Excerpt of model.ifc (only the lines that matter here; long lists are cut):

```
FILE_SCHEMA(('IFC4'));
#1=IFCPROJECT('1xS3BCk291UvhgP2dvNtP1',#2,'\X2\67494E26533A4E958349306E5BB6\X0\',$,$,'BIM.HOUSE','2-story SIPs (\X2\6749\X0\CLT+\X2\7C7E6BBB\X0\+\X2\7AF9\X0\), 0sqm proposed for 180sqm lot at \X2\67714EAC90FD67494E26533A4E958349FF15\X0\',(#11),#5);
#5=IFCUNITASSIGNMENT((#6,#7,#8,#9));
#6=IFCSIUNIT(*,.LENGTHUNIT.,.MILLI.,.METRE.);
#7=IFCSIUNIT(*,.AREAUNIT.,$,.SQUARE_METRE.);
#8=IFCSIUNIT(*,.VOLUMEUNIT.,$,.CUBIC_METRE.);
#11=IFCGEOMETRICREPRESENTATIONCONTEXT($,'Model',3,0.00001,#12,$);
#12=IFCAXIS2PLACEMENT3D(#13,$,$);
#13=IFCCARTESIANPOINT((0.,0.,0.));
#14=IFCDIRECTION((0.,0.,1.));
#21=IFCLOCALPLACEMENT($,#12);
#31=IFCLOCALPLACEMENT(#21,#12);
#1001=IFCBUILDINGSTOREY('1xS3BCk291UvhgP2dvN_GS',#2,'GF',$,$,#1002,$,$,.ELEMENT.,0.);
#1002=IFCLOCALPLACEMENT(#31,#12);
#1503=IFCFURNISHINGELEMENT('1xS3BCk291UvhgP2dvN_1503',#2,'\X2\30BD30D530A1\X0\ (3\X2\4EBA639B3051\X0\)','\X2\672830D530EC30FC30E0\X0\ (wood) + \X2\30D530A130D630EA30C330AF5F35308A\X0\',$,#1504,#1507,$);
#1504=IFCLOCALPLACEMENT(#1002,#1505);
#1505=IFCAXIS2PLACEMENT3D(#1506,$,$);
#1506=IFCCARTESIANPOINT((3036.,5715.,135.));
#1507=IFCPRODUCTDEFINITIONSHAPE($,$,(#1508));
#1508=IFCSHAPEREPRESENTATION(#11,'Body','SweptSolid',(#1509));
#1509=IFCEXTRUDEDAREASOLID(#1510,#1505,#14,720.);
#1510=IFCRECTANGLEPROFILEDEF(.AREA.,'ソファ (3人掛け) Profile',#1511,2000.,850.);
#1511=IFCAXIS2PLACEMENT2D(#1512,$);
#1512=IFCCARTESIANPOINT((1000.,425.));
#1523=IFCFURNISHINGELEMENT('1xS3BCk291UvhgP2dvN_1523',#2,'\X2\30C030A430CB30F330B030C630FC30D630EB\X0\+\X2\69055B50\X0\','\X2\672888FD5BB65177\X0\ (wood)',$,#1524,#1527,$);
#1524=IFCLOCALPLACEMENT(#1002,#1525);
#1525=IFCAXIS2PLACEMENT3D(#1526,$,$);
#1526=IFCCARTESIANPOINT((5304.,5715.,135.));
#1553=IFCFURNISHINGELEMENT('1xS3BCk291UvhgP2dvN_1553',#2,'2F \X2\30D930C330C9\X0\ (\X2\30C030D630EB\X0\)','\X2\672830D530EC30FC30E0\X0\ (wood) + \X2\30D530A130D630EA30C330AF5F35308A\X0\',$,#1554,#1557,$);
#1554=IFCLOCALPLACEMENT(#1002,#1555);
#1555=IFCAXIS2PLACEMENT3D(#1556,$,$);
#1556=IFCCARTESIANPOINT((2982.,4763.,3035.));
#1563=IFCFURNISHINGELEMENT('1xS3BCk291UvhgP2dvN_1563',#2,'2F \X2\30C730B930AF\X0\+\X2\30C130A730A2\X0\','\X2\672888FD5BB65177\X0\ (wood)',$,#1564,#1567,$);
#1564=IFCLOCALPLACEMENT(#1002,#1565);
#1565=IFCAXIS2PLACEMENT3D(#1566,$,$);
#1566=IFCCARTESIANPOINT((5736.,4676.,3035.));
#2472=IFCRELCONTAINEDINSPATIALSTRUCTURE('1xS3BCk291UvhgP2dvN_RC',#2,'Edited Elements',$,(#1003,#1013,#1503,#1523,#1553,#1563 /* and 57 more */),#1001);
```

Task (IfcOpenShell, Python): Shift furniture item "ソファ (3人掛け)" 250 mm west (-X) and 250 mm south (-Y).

```python
import ifcopenshell
import ifcopenshell.api.geometry
import ifcopenshell.util.placement
import ifcopenshell.util.unit

model = ifcopenshell.open("model.ifc")
unit_scale = ifcopenshell.util.unit.calculate_unit_scale(model)

item = model.by_guid("1xS3BCk291UvhgP2dvN_1503")
matrix = ifcopenshell.util.placement.get_local_placement(item.ObjectPlacement)
matrix[0, 3] -= 0.25 / unit_scale
matrix[1, 3] -= 0.25 / unit_scale
ifcopenshell.api.geometry.edit_object_placement(model, product=item, matrix=matrix, is_si=False)

print(ifcopenshell.util.placement.get_local_placement(item.ObjectPlacement).round(3) + 0.0)

model.write("model_edited.ifc")
```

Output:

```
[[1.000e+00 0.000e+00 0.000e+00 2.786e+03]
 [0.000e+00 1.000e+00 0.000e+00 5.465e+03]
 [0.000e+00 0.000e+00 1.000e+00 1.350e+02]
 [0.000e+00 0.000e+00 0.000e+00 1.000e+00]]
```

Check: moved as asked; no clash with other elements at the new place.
